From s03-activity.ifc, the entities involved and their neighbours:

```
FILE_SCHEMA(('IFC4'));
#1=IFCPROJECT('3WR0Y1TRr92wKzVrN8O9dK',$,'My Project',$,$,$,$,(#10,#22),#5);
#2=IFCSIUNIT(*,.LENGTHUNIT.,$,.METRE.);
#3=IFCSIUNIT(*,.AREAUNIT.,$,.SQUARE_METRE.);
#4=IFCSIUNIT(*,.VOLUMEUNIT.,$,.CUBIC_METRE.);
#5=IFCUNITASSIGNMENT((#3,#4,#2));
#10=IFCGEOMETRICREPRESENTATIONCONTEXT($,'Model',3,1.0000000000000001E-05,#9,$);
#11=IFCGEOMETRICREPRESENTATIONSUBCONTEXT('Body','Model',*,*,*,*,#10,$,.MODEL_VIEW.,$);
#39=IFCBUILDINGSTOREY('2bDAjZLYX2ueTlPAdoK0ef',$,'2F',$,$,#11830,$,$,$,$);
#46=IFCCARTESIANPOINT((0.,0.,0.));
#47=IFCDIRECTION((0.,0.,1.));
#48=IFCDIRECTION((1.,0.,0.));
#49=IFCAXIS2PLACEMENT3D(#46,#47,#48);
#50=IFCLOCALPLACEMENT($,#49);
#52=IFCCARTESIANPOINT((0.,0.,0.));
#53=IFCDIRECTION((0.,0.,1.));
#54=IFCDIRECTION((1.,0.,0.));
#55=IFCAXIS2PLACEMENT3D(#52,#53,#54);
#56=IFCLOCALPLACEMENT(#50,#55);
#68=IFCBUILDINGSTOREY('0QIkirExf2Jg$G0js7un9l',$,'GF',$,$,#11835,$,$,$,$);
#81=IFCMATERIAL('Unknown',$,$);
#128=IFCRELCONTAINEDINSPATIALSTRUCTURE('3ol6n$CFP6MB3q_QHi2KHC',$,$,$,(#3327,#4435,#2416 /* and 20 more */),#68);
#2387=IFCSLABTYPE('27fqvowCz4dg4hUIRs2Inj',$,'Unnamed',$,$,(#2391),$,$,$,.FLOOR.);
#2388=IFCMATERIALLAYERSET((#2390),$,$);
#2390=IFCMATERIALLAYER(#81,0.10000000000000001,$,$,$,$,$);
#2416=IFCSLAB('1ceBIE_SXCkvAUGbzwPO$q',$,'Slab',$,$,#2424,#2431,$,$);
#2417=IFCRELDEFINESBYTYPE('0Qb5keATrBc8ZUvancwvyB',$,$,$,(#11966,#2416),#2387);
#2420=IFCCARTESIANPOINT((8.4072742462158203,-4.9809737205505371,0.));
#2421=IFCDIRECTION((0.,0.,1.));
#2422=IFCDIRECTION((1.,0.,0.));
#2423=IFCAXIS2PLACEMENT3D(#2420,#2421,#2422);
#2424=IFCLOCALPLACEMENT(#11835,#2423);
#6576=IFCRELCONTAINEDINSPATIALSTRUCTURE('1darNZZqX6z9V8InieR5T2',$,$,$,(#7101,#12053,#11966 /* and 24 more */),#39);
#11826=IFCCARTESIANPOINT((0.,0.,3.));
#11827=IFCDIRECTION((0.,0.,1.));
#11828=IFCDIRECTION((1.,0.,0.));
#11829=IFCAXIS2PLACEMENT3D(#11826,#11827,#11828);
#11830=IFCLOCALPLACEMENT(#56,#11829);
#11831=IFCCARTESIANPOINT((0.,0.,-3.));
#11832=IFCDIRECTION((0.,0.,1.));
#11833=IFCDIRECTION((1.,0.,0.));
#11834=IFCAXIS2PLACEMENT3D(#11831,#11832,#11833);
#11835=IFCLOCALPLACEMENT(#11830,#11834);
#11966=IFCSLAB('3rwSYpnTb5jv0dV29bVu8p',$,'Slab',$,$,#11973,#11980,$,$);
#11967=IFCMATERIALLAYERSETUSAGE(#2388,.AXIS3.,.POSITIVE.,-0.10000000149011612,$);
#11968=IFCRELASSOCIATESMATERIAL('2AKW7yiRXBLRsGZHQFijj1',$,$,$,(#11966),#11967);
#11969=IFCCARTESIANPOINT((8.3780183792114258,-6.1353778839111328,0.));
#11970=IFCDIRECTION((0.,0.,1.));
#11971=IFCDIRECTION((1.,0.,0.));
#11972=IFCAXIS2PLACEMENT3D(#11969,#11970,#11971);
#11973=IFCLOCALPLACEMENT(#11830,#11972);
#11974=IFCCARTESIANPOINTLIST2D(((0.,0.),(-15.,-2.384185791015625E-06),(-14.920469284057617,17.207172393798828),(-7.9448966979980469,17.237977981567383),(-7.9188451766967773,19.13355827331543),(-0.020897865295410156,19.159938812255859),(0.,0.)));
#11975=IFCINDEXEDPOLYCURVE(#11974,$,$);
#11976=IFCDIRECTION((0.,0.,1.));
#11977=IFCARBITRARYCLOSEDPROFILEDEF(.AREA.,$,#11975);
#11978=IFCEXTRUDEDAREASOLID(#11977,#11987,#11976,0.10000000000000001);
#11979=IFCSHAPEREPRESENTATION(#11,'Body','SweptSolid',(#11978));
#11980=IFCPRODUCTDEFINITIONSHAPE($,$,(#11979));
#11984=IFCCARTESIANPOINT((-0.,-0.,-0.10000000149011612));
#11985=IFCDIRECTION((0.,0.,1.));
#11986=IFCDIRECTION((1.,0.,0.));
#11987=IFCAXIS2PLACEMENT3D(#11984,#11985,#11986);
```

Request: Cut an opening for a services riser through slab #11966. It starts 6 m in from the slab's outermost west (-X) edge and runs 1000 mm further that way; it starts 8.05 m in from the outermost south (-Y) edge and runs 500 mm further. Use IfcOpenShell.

```python
import numpy as np
import ifcopenshell
import ifcopenshell.api.feature
import ifcopenshell.api.geometry
import ifcopenshell.api.root
import ifcopenshell.geom
import ifcopenshell.util.placement
import ifcopenshell.util.representation
import ifcopenshell.util.shape
import ifcopenshell.util.unit

model = ifcopenshell.open("s03-activity.ifc")
unit_scale = ifcopenshell.util.unit.calculate_unit_scale(model)
settings = ifcopenshell.geom.settings()


def volume(element):
    """Net volume in cubic metres, openings subtracted."""
    shape = ifcopenshell.geom.create_shape(settings, element)
    return ifcopenshell.util.shape.get_volume(shape.geometry)


slab = model.by_id(11966)
before = volume(slab)

# Extent in the slab's own axes, in metres. The edges named are its -X and -Y sides.
slab_shape = ifcopenshell.geom.create_shape(settings, slab)
vertices = ifcopenshell.util.shape.get_vertices(slab_shape.geometry)
x_min, y_min, bottom = vertices.min(axis=0)
top = vertices[:, 2].max()

opening = ifcopenshell.api.root.create_entity(model, ifc_class="IfcOpeningElement", name="Services riser opening", predefined_type="OPENING")
context = ifcopenshell.util.representation.get_context(model, "Model", "Body", "MODEL_VIEW")
width, depth = 1, 0.5
outline = [(0.0, 0.0), (width, 0.0), (width, depth), (0.0, depth), (0.0, 0.0)]
# Overshoot both faces by 50 mm so the cut is clean.
shape = ifcopenshell.api.geometry.add_slab_representation(
    model, context=context, depth=top - bottom + 0.1, polyline=outline
)
ifcopenshell.api.geometry.assign_representation(model, product=opening, representation=shape)

matrix = ifcopenshell.util.placement.get_local_placement(slab.ObjectPlacement)
matrix[:, 3] = matrix @ np.append(np.array([x_min + 6, y_min + 8.05, bottom - 0.05]) / unit_scale, 1.0)
ifcopenshell.api.geometry.edit_object_placement(model, product=opening, matrix=matrix, is_si=False)
ifcopenshell.api.feature.add_feature(model, feature=opening, element=slab)

after = volume(slab)

print(f"slab volume {before:.3f} -> {after:.3f} m3")

model.write("s03-activity_v2.ifc")
```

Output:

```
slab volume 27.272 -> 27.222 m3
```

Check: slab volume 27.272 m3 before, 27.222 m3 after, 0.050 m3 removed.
